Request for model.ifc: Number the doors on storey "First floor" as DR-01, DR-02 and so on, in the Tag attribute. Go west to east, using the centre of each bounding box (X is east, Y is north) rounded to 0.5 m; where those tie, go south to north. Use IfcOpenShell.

First a look at what the model holds.

```python
import ifcopenshell
import ifcopenshell.util.element
import ifcopenshell.util.placement

model = ifcopenshell.open("model.ifc")
print(model.schema)
storey = next(s for s in model.by_type("IfcBuildingStorey") if s.Name == "First floor")
doors = [e for e in ifcopenshell.util.element.get_decomposition(storey) if e.is_a("IfcDoor")]
for e in sorted(doors, key=lambda e: e.id()):
    origin = ifcopenshell.util.placement.get_local_placement(e.ObjectPlacement)[:3, 3]
    print(e.id(), e.Tag, e.Name, origin.round(2) + 0.0, sep=" | ")
```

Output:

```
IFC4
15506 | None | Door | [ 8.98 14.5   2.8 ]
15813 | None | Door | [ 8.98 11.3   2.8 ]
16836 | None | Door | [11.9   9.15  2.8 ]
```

```python
import ifcopenshell
import ifcopenshell.geom
import ifcopenshell.util.element
import ifcopenshell.util.shape

model = ifcopenshell.open("model.ifc")
settings = ifcopenshell.geom.settings()
settings.set("use-world-coords", True)


def centre(element):
    shape = ifcopenshell.geom.create_shape(settings, element)
    return ifcopenshell.util.shape.get_bbox_centroid(shape.geometry)


storey = next(s for s in model.by_type("IfcBuildingStorey") if s.Name == "First floor")
doors = [e for e in ifcopenshell.util.element.get_decomposition(storey) if e.is_a("IfcDoor")]

# Insertion points can sit at a corner or the storey origin, so sort by the geometry (in metres).
centres = {e: centre(e) for e in doors}
doors.sort(key=lambda e: (round(centres[e][0] / 0.5), centres[e][1]))

for i, e in enumerate(doors, start=1):
    number = f"DR-{i:02d}"
    e.Tag = number
    print(e.id(), number)

model.write("model_rev.ifc")
```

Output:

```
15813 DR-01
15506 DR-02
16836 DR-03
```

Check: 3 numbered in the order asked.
